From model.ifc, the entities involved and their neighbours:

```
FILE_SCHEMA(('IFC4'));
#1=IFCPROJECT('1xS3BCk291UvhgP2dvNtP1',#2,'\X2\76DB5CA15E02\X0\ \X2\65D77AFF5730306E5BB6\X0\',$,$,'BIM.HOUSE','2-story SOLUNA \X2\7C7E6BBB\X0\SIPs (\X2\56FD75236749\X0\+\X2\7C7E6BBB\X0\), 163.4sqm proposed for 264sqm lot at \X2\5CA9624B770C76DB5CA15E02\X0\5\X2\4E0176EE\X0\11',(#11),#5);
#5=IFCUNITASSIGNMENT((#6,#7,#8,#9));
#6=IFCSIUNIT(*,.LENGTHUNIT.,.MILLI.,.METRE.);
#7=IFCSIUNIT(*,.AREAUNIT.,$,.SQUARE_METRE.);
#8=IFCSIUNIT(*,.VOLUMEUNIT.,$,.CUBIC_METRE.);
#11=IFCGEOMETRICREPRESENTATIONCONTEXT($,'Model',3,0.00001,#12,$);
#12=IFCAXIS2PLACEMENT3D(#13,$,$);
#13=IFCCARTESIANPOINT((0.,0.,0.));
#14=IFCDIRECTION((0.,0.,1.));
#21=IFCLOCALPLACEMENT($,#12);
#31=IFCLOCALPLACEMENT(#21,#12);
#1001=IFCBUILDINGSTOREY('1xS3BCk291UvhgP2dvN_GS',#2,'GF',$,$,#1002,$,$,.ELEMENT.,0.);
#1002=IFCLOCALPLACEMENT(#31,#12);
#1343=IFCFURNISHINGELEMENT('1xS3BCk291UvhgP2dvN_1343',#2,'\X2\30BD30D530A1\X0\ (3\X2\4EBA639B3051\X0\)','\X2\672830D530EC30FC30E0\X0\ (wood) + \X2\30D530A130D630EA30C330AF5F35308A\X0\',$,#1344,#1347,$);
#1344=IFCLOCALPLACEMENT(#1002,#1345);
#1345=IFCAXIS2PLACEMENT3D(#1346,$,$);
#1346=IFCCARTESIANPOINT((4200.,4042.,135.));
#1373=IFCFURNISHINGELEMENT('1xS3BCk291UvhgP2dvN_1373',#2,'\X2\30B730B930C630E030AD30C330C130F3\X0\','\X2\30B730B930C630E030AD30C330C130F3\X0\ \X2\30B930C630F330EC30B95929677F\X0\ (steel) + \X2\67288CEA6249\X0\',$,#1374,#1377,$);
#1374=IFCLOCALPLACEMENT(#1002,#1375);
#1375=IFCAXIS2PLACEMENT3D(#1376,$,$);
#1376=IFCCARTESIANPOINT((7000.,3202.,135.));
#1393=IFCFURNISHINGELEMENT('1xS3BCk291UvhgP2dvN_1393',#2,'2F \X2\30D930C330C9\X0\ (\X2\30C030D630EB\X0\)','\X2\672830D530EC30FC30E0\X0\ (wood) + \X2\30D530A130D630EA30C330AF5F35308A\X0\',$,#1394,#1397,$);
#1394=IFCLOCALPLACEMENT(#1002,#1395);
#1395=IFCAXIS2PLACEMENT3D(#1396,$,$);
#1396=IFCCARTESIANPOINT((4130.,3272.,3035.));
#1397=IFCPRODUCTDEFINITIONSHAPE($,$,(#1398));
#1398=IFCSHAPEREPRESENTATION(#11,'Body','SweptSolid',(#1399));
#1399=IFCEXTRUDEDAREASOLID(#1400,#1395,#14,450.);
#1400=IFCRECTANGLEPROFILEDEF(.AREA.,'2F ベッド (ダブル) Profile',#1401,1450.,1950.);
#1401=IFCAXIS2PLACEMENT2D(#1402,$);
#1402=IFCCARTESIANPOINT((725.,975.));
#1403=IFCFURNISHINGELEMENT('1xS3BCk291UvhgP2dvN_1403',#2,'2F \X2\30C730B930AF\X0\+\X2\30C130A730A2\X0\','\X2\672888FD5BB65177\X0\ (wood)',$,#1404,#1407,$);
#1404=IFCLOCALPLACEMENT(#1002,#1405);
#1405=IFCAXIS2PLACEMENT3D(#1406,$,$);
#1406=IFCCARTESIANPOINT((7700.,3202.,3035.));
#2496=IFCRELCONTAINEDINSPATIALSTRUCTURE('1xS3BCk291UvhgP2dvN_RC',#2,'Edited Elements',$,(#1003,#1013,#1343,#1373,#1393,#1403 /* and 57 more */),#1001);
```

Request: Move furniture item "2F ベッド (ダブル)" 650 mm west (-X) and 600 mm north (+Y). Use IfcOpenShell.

```python
import ifcopenshell
import ifcopenshell.api.geometry
import ifcopenshell.util.placement
import ifcopenshell.util.unit

model = ifcopenshell.open("model.ifc")
unit_scale = ifcopenshell.util.unit.calculate_unit_scale(model)

item = model.by_guid("1xS3BCk291UvhgP2dvN_1393")
matrix = ifcopenshell.util.placement.get_local_placement(item.ObjectPlacement)
matrix[0, 3] -= 0.65 / unit_scale
matrix[1, 3] += 0.6 / unit_scale
ifcopenshell.api.geometry.edit_object_placement(model, product=item, matrix=matrix, is_si=False)

print(ifcopenshell.util.placement.get_local_placement(item.ObjectPlacement).round(3) + 0.0)

model.write("model_edited.ifc")
```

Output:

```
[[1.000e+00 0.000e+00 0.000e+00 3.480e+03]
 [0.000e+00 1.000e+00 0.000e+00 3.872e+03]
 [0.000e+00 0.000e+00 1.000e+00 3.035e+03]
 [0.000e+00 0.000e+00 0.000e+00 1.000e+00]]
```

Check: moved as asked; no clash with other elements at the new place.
